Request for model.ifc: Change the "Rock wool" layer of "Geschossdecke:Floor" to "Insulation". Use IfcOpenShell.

First a look at what the model holds.

```python
import ifcopenshell
import ifcopenshell.util.element

model = ifcopenshell.open("model.ifc")
print(model.schema)
for layer_set in model.by_type("IfcMaterialLayerSet"):
    if layer_set.LayerSetName == "Geschossdecke:Floor":
        for layer in layer_set.MaterialLayers:
            print(layer.id(), layer.Material and layer.Material.Name, layer.LayerThickness, sep=" | ")
        print(len(ifcopenshell.util.element.get_elements_by_material(model, layer_set)), "elements and types use it")
print(sorted(m.Name for m in model.by_type("IfcMaterial") if m.Name)[:60])
```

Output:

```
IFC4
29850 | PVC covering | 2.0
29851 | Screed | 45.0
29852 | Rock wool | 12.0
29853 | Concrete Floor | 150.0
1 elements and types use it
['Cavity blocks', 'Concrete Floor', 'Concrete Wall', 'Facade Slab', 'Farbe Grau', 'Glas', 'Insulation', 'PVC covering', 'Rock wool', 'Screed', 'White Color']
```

```python
import ifcopenshell
import ifcopenshell.api.material

model = ifcopenshell.open("model.ifc")

layer_set = next(s for s in model.by_type("IfcMaterialLayerSet") if s.LayerSetName == "Geschossdecke:Floor")
layer = next(l for l in layer_set.MaterialLayers if l.Material and l.Material.Name == "Rock wool")
material = next(m for m in model.by_type("IfcMaterial") if m.Name == "Insulation")

# Point this one layer at the other material; renaming the old one would change it everywhere.
ifcopenshell.api.material.edit_layer(model, layer=layer, attributes={}, material=material)

print([l.Material.Name if l.Material else None for l in layer_set.MaterialLayers])

model.write("model_v2.ifc")
```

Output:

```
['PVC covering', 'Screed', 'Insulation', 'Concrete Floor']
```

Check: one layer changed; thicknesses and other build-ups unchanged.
